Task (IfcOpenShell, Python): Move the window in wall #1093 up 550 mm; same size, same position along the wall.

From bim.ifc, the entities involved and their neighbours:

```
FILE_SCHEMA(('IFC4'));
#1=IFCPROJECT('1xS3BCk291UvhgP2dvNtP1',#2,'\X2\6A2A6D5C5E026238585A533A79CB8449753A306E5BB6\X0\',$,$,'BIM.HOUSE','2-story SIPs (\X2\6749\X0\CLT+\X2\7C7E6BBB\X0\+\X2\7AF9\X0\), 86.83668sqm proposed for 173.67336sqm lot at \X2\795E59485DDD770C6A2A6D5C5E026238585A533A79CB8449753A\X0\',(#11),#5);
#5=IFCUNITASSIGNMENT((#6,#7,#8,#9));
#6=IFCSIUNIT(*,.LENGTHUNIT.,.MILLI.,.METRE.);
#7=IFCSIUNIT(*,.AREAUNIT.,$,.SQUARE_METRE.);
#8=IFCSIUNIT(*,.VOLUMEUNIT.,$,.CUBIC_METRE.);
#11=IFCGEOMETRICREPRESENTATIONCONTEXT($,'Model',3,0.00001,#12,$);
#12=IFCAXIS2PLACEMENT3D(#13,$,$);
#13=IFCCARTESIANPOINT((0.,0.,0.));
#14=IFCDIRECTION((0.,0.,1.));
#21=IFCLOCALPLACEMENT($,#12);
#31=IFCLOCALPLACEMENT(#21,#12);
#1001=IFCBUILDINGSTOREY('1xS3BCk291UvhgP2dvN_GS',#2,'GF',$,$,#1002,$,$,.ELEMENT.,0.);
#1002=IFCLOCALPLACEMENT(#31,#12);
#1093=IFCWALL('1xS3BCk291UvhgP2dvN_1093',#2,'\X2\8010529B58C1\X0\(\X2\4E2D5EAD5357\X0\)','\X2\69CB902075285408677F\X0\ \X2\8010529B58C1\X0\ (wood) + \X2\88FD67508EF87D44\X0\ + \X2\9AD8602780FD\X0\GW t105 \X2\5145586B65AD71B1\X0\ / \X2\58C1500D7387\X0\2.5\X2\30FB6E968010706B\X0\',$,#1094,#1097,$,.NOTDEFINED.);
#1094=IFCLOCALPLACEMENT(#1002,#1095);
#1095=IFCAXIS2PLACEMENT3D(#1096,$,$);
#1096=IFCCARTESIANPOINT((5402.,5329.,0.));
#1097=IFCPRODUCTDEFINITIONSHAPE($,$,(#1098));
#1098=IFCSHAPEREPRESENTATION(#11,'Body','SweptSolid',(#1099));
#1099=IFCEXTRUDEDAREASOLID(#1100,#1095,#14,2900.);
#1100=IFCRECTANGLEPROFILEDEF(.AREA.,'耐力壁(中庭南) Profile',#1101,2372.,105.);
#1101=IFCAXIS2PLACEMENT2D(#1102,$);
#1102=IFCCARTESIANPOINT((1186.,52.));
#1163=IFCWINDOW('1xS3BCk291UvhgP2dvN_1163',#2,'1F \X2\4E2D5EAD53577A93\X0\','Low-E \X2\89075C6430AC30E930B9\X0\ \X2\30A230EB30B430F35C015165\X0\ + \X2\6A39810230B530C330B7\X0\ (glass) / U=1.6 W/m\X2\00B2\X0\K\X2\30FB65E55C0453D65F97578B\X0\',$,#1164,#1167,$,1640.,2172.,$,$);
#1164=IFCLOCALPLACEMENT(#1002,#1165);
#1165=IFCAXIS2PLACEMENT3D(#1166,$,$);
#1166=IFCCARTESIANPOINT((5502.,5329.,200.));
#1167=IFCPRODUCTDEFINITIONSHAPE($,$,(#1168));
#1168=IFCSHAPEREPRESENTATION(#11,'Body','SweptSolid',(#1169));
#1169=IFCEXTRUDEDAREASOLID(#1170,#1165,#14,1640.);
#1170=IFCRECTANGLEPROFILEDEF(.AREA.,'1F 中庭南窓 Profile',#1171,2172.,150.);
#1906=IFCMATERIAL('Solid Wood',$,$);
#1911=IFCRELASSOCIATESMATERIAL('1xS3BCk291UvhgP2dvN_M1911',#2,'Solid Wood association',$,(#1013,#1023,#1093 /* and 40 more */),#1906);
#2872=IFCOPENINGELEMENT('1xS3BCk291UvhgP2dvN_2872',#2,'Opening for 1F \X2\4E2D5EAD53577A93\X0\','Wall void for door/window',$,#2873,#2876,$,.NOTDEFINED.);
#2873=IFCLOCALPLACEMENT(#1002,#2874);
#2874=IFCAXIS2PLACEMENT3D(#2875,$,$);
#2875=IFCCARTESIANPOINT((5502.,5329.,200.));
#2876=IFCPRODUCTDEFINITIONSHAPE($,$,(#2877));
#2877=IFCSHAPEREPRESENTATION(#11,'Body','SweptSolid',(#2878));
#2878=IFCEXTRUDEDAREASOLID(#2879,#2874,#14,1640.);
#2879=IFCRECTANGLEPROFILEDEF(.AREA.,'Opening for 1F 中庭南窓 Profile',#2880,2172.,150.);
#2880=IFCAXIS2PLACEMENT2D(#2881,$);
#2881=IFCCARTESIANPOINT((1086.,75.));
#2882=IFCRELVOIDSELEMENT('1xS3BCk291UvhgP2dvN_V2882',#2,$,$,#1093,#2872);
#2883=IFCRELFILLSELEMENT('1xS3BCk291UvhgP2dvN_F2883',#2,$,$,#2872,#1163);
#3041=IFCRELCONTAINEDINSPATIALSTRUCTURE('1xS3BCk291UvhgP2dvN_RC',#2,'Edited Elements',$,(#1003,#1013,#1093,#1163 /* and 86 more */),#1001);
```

```python
import numpy as np
import ifcopenshell
import ifcopenshell.api.geometry
import ifcopenshell.util.placement
import ifcopenshell.util.unit

model = ifcopenshell.open("bim.ifc")
unit_scale = ifcopenshell.util.unit.calculate_unit_scale(model)

window = model.by_id(1163)
opening = window.FillsVoids[0].RelatingOpeningElement
dz = 550.0

shift = np.array([0.0, 0.0, dz])
# The window is not placed relative to its opening, so move both.
for product in (opening, window):
    matrix = ifcopenshell.util.placement.get_local_placement(product.ObjectPlacement)
    matrix[:3, 3] += shift
    ifcopenshell.api.geometry.edit_object_placement(model, product=product, matrix=matrix, is_si=False)

print(f"moved by {dz * unit_scale:+.3f} m")

model.write("bim_edited.ifc")
```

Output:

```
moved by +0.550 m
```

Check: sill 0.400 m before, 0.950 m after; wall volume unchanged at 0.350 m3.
